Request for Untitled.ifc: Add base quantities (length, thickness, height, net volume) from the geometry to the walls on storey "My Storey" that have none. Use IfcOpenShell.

First a look at what the model holds.

```python
import ifcopenshell
import ifcopenshell.util.element
import ifcopenshell.util.unit

model = ifcopenshell.open("Untitled.ifc")
print(model.schema)
for unit_type in ("LENGTHUNIT", "AREAUNIT", "VOLUMEUNIT"):
    print(unit_type, ifcopenshell.util.unit.calculate_unit_scale(model, unit_type))
storey = next(s for s in model.by_type("IfcBuildingStorey") if s.Name == "My Storey")
walls = [e for e in ifcopenshell.util.element.get_decomposition(storey) if e.is_a("IfcWall")]
for e in sorted(walls, key=lambda e: e.id()):
    print(e.id(), e.is_a(), e.Name, list(ifcopenshell.util.element.get_psets(e, qtos_only=True)), sep=" | ")
```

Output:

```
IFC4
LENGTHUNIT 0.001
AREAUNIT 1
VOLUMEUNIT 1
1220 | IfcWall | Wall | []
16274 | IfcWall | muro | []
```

```python
import ifcopenshell
import ifcopenshell.api.pset
import ifcopenshell.geom
import ifcopenshell.util.element
import ifcopenshell.util.shape
import ifcopenshell.util.unit

model = ifcopenshell.open("Untitled.ifc")
unit_scale = ifcopenshell.util.unit.calculate_unit_scale(model)
volume_scale = ifcopenshell.util.unit.calculate_unit_scale(model, "VOLUMEUNIT")
settings = ifcopenshell.geom.settings()

storey = next(s for s in model.by_type("IfcBuildingStorey") if s.Name == "My Storey")
walls = [e for e in ifcopenshell.util.element.get_decomposition(storey) if e.is_a("IfcWall")]

for e in sorted(walls, key=lambda e: e.id()):
    if ifcopenshell.util.element.get_psets(e, qtos_only=True, should_inherit=False):
        continue
    # Geometry comes back in metres, in the element's own axes.
    shape = ifcopenshell.geom.create_shape(settings, e)
    values = {
        "Length": ifcopenshell.util.shape.get_x(shape.geometry) / unit_scale,
        "Width": ifcopenshell.util.shape.get_y(shape.geometry) / unit_scale,
        "Height": ifcopenshell.util.shape.get_z(shape.geometry) / unit_scale,
        "NetVolume": ifcopenshell.util.shape.get_volume(shape.geometry) / volume_scale,
    }
    qto = ifcopenshell.api.pset.add_qto(model, product=e, name="Qto_WallBaseQuantities")
    ifcopenshell.api.pset.edit_qto(model, qto=qto, properties=values)
    print(e.id(), {k: round(v, 3) for k, v in values.items()})

model.write("Untitled_updated.ifc")
```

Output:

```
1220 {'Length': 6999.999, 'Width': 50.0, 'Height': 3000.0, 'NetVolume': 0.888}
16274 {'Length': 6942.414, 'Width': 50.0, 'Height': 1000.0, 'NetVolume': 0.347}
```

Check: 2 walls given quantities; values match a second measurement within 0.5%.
